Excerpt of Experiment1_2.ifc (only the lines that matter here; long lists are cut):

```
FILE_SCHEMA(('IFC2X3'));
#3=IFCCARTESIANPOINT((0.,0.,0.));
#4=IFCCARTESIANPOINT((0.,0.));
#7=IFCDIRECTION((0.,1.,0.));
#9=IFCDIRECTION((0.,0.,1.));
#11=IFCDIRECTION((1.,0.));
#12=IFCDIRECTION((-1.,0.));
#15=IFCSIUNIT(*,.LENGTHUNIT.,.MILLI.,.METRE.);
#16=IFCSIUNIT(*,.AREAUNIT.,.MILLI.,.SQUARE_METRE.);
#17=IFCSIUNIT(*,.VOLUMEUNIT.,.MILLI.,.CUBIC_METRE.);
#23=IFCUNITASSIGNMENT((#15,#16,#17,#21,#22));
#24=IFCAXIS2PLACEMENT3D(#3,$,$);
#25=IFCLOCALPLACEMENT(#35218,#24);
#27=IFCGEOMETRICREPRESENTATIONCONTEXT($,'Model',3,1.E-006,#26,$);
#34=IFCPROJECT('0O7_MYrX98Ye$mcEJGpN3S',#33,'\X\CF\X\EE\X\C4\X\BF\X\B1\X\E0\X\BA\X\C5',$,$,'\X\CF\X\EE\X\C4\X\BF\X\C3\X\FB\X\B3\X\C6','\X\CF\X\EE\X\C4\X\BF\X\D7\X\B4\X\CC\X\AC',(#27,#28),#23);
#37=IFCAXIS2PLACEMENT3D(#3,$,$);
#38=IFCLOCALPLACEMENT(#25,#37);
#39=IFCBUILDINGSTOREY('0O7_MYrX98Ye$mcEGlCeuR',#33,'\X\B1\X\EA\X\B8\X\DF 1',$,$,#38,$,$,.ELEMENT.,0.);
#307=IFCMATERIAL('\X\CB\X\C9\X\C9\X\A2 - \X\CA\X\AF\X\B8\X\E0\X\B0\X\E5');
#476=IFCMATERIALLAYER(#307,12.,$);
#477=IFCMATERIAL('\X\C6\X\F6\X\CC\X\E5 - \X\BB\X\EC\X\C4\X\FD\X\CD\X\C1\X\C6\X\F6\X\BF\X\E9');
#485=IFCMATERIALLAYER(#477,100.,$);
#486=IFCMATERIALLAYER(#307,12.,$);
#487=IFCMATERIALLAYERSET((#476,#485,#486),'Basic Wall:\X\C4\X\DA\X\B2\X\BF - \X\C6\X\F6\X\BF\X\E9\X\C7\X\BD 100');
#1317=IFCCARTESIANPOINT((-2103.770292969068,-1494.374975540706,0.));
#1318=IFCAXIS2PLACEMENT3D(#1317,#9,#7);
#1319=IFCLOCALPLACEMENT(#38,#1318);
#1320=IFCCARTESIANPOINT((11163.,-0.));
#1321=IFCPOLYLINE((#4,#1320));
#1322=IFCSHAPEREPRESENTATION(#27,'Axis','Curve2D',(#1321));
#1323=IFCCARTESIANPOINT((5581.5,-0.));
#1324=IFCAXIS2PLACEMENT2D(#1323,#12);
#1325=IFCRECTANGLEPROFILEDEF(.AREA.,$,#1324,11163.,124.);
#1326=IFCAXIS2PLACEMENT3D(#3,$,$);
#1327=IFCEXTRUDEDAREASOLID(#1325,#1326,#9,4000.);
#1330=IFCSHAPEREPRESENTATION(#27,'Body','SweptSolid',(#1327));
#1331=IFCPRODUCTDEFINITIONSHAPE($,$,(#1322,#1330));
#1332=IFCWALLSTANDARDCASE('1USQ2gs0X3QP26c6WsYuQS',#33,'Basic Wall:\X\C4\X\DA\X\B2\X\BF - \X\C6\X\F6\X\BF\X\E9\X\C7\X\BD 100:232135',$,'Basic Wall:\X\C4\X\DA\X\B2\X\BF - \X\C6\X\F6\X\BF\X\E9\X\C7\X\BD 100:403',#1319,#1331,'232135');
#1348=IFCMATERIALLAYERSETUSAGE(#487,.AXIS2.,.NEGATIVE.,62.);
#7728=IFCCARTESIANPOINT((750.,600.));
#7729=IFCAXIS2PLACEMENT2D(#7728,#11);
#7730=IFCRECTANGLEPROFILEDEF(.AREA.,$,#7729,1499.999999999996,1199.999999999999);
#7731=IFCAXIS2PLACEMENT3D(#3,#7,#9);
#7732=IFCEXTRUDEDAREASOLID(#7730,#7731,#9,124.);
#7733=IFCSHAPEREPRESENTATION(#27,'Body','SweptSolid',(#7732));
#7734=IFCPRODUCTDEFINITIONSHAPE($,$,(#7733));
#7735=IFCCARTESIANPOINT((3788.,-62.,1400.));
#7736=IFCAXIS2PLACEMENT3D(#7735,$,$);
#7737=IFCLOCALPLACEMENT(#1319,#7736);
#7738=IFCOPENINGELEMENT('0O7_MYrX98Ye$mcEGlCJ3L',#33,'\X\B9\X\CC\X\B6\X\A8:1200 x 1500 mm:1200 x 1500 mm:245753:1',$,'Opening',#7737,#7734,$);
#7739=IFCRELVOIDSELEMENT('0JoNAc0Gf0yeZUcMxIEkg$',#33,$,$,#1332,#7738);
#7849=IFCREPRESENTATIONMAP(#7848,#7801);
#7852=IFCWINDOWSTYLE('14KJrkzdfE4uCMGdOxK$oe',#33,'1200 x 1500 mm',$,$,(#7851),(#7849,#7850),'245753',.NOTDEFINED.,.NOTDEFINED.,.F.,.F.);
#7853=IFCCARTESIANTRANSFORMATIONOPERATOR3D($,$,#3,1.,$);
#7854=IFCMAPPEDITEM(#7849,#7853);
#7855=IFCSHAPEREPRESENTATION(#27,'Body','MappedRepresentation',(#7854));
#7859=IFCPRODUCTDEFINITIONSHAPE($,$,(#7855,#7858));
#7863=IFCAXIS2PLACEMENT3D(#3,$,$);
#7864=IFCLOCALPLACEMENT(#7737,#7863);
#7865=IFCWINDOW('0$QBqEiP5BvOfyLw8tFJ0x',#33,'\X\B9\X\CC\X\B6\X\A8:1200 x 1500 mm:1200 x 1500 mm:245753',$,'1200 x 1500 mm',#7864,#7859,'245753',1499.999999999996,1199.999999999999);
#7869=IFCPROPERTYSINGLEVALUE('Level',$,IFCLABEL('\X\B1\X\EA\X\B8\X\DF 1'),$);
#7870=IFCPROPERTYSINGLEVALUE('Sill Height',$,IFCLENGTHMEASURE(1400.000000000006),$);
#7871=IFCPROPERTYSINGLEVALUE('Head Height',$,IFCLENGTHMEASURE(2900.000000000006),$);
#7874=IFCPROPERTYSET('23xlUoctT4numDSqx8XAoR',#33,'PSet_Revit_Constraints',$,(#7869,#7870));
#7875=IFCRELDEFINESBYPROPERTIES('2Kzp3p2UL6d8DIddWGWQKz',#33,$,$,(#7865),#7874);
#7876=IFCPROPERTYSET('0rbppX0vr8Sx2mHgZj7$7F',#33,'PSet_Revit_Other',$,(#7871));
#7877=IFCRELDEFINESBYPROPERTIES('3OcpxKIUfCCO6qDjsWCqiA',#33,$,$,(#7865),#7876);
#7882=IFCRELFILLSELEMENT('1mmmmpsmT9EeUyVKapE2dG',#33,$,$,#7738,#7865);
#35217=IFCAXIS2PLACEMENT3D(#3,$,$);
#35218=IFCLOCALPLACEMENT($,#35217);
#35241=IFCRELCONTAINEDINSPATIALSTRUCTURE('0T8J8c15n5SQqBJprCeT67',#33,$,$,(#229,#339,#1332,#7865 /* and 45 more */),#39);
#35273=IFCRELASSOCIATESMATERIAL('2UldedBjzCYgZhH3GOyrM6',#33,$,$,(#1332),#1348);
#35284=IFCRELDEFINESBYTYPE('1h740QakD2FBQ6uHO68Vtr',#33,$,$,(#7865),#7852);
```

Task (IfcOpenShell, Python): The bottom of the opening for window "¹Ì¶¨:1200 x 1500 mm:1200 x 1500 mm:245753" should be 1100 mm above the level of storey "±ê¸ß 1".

```python
import numpy as np
import ifcopenshell
import ifcopenshell.api.geometry
import ifcopenshell.api.pset
import ifcopenshell.geom
import ifcopenshell.util.element
import ifcopenshell.util.placement
import ifcopenshell.util.shape
import ifcopenshell.util.unit

model = ifcopenshell.open("Experiment1_2.ifc")
unit_scale = ifcopenshell.util.unit.calculate_unit_scale(model)

window = model.by_guid("0$QBqEiP5BvOfyLw8tFJ0x")
opening = window.FillsVoids[0].RelatingOpeningElement
storey = ifcopenshell.util.element.get_container(window, ifc_class="IfcBuildingStorey")
level = ifcopenshell.util.placement.get_local_placement(storey.ObjectPlacement)[2, 3]

# The opening's origin need not be at the sill, so measure its lowest point.
shape = ifcopenshell.geom.create_shape(ifcopenshell.geom.settings(), opening)
bottom = ifcopenshell.util.shape.get_shape_bottom_elevation(shape, shape.geometry) / unit_scale
dz = level + 1.1 / unit_scale - bottom

shift = np.array([0.0, 0.0, dz])
# The window is placed relative to its opening, so it follows when the opening moves.
matrix = ifcopenshell.util.placement.get_local_placement(opening.ObjectPlacement)
matrix[:3, 3] += shift
ifcopenshell.api.geometry.edit_object_placement(
    model, product=opening, matrix=matrix, is_si=False, should_transform_children=True
)

# Keep the stored heights in step.
pset = model.by_id(ifcopenshell.util.element.get_pset(window, "PSet_Revit_Constraints", should_inherit=False)["id"])
ifcopenshell.api.pset.edit_pset(model, pset=pset, properties={
    "Sill Height": model.create_entity("IfcLengthMeasure", ifcopenshell.util.element.get_pset(window, "PSet_Revit_Constraints", "Sill Height") + dz),
})
pset = model.by_id(ifcopenshell.util.element.get_pset(window, "PSet_Revit_Other", should_inherit=False)["id"])
ifcopenshell.api.pset.edit_pset(model, pset=pset, properties={
    "Head Height": model.create_entity("IfcLengthMeasure", ifcopenshell.util.element.get_pset(window, "PSet_Revit_Other", "Head Height") + dz),
})

print(f"moved by {dz * unit_scale:+.3f} m")

model.write("Experiment1_2_v2.ifc")
```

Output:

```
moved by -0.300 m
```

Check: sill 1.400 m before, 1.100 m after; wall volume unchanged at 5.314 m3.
